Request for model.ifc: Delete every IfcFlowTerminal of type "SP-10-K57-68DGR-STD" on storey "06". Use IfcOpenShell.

First a look at what the model holds.

```python
import ifcopenshell
import ifcopenshell.util.element

model = ifcopenshell.open("model.ifc")
print(model.schema)
storey = next(s for s in model.by_type("IfcBuildingStorey") if s.Name == "06")
terminals = [e for e in ifcopenshell.util.element.get_decomposition(storey) if e.is_a("IfcFlowTerminal")]
seen = {}
for e in terminals:
    element_type = ifcopenshell.util.element.get_type(e)
    name = element_type.Name if element_type not in (None, e) else None
    seen[name] = seen.get(name, 0) + 1
for name, count in sorted(seen.items(), key=str):
    print(count, "x", name)
```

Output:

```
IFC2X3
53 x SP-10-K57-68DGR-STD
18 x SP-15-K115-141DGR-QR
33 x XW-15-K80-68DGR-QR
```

```python
import ifcopenshell
import ifcopenshell.api.root
import ifcopenshell.util.element

model = ifcopenshell.open("model.ifc")

storey = next(s for s in model.by_type("IfcBuildingStorey") if s.Name == "06")
terminals = [e for e in ifcopenshell.util.element.get_decomposition(storey) if e.is_a("IfcFlowTerminal")]
targets = [e for e in terminals if (t := ifcopenshell.util.element.get_type(e)) not in (None, e) and t.Name == "SP-10-K57-68DGR-STD"]

for e in targets:
    ifcopenshell.api.root.remove_product(model, product=e)
print(len(targets), "removed")

model.write("model_updated.ifc")
```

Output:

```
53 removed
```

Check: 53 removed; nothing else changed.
